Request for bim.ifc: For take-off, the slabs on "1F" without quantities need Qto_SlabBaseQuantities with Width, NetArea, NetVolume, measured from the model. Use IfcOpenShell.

First a look at what the model holds.

```python
import ifcopenshell
import ifcopenshell.util.element
import ifcopenshell.util.unit

model = ifcopenshell.open("bim.ifc")
print(model.schema)
for unit_type in ("LENGTHUNIT", "AREAUNIT", "VOLUMEUNIT"):
    print(unit_type, ifcopenshell.util.unit.calculate_unit_scale(model, unit_type))
storey = next(s for s in model.by_type("IfcBuildingStorey") if s.Name == "1F")
slabs = [e for e in ifcopenshell.util.element.get_decomposition(storey) if e.is_a("IfcSlab")]
for e in sorted(slabs, key=lambda e: e.id()):
    print(e.id(), e.is_a(), e.Name, list(ifcopenshell.util.element.get_psets(e, qtos_only=True)), sep=" | ")
```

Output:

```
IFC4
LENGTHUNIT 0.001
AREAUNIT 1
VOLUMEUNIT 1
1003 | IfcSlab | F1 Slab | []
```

```python
import ifcopenshell
import ifcopenshell.api.pset
import ifcopenshell.geom
import ifcopenshell.util.element
import ifcopenshell.util.shape
import ifcopenshell.util.unit

model = ifcopenshell.open("bim.ifc")
unit_scale = ifcopenshell.util.unit.calculate_unit_scale(model)
area_scale = ifcopenshell.util.unit.calculate_unit_scale(model, "AREAUNIT")
volume_scale = ifcopenshell.util.unit.calculate_unit_scale(model, "VOLUMEUNIT")
settings = ifcopenshell.geom.settings()

storey = next(s for s in model.by_type("IfcBuildingStorey") if s.Name == "1F")
slabs = [e for e in ifcopenshell.util.element.get_decomposition(storey) if e.is_a("IfcSlab")]

for e in sorted(slabs, key=lambda e: e.id()):
    if ifcopenshell.util.element.get_psets(e, qtos_only=True, should_inherit=False):
        continue
    # Geometry comes back in metres, in the element's own axes.
    shape = ifcopenshell.geom.create_shape(settings, e)
    values = {
        "Width": ifcopenshell.util.shape.get_z(shape.geometry) / unit_scale,
        "NetArea": ifcopenshell.util.shape.get_footprint_area(shape.geometry) / area_scale,
        "NetVolume": ifcopenshell.util.shape.get_volume(shape.geometry) / volume_scale,
    }
    qto = ifcopenshell.api.pset.add_qto(model, product=e, name="Qto_SlabBaseQuantities")
    ifcopenshell.api.pset.edit_qto(model, qto=qto, properties=values)
    print(e.id(), {k: round(v, 3) for k, v in values.items()})

model.write("bim_rev.ifc")
```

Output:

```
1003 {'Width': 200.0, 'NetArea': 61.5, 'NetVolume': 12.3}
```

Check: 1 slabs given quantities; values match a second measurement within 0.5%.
